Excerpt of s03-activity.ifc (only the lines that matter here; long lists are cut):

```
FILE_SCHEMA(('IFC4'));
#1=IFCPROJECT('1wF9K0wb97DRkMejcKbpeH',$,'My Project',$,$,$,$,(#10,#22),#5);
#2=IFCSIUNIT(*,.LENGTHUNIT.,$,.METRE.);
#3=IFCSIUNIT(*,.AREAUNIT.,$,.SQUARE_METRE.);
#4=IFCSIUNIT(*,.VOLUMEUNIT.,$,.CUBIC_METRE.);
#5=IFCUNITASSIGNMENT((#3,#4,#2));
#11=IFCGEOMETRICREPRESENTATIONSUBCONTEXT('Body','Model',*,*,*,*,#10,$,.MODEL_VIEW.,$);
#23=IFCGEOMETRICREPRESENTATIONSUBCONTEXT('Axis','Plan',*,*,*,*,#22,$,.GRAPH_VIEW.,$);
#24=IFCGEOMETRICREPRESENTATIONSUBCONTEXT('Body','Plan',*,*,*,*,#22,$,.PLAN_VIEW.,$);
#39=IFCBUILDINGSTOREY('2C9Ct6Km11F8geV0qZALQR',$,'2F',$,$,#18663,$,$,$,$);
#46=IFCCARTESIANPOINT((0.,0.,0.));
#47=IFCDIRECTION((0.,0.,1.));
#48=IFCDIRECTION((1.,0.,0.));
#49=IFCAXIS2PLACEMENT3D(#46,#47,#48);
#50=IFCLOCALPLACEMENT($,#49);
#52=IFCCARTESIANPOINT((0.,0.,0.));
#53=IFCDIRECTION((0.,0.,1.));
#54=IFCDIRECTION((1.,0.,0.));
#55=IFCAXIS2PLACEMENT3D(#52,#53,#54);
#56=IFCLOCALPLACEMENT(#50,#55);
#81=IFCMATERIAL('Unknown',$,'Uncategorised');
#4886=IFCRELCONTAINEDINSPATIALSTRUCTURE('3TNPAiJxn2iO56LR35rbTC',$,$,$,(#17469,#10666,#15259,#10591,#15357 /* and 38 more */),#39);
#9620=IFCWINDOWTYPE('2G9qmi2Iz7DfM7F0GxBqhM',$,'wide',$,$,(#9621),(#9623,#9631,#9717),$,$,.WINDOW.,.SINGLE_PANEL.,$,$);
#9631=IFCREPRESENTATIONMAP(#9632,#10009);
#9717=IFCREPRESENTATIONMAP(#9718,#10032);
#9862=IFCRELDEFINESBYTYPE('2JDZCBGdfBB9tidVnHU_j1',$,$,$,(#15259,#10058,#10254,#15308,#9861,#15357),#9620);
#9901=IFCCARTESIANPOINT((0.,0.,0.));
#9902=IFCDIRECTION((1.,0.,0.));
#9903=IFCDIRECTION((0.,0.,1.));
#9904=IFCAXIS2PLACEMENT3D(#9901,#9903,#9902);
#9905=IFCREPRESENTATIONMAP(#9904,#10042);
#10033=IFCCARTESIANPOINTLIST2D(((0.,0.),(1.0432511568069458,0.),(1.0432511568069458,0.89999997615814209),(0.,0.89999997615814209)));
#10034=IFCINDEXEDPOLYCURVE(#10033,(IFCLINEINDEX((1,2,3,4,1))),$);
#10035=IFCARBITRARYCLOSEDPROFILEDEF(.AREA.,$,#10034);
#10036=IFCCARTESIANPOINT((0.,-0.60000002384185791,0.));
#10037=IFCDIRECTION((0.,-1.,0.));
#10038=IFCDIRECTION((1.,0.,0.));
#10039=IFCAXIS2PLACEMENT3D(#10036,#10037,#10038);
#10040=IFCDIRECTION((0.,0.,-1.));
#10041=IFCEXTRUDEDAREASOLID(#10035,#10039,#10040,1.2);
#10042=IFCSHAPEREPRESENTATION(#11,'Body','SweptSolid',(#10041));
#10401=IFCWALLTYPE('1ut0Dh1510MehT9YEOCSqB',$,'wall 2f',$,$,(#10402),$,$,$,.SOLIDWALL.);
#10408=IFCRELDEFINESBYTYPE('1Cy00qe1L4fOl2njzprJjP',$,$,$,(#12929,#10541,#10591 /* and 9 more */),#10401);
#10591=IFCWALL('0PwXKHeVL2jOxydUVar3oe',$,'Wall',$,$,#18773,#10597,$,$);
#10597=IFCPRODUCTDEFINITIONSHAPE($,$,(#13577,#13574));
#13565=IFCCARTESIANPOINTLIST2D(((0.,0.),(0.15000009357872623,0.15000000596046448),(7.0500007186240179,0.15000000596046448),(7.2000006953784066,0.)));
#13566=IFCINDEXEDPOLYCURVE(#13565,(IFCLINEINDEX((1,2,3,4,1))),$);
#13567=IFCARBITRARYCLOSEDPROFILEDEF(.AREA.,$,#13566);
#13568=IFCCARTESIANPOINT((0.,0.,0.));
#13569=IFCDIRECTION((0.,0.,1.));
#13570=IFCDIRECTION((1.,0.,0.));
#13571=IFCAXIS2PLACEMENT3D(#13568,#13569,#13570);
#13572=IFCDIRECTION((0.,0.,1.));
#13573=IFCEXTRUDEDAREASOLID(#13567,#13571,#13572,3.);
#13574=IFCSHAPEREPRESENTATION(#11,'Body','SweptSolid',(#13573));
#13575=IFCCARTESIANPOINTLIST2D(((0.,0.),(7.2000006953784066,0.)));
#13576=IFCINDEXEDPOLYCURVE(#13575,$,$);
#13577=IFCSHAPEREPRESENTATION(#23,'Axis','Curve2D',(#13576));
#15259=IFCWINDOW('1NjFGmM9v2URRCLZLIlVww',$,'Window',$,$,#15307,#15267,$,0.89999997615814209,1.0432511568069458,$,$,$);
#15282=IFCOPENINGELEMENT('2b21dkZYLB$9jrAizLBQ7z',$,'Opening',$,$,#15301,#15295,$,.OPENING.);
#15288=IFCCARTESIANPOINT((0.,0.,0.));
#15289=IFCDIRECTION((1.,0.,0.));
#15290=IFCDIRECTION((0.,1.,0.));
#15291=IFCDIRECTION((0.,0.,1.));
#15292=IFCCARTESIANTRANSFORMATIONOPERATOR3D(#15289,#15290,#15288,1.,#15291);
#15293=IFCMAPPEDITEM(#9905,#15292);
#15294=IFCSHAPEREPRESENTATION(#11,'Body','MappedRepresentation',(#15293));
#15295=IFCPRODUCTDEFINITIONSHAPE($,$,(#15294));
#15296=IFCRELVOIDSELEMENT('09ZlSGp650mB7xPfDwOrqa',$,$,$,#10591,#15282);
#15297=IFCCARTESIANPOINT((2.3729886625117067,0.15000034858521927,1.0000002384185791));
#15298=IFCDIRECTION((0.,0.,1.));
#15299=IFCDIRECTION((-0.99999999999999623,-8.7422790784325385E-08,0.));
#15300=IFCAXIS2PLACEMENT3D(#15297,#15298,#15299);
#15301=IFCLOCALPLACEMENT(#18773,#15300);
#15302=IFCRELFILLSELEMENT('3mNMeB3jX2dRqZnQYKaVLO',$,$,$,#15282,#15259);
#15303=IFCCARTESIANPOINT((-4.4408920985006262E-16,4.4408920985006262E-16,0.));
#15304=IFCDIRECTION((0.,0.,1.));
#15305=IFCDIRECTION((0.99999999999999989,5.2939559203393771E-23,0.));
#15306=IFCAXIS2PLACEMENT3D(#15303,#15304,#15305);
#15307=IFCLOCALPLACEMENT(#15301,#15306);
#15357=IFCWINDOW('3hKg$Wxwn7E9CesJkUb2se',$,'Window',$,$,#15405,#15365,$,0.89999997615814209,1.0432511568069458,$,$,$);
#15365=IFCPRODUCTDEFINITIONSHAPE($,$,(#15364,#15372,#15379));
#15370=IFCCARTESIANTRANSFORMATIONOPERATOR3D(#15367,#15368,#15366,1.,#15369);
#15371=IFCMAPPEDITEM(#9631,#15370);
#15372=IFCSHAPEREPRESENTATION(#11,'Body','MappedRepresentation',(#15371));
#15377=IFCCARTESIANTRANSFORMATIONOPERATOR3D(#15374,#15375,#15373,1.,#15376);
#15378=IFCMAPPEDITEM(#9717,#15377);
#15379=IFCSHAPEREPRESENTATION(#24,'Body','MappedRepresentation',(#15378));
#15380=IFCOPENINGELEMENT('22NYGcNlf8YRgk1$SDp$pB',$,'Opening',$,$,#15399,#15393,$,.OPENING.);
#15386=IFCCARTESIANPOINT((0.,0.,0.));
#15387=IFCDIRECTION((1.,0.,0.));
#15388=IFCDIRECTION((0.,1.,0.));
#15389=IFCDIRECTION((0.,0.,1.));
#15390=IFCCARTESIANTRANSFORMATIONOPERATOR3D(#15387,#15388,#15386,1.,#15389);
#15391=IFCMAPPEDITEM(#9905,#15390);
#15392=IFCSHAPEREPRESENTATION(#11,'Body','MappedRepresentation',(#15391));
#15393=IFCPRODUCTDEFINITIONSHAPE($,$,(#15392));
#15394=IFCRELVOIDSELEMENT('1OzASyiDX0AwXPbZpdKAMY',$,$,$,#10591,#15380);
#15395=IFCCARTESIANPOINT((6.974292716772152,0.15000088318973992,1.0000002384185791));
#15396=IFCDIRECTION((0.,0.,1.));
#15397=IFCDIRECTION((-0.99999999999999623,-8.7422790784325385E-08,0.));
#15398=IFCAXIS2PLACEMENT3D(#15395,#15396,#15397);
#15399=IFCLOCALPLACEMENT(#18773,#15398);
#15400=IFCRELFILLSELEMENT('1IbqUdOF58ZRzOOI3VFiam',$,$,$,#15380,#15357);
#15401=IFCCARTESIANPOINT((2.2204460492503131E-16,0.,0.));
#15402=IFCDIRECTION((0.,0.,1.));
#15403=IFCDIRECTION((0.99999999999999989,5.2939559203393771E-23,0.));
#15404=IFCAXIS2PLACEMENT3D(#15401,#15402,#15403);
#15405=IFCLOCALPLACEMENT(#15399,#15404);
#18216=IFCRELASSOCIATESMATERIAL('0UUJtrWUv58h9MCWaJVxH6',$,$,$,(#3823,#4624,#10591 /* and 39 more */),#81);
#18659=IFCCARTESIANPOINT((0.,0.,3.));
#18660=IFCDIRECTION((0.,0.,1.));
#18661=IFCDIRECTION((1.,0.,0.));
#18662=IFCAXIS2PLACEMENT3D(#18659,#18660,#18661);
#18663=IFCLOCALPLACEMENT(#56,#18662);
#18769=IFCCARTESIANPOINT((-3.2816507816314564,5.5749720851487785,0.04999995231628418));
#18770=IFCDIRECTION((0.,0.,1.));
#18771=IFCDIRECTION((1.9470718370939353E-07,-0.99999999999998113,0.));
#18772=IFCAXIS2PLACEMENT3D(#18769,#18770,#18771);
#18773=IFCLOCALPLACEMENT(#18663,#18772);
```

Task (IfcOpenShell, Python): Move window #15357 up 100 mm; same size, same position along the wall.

```python
import numpy as np
import ifcopenshell
import ifcopenshell.api.geometry
import ifcopenshell.util.placement
import ifcopenshell.util.unit

model = ifcopenshell.open("s03-activity.ifc")
unit_scale = ifcopenshell.util.unit.calculate_unit_scale(model)

window = model.by_id(15357)
opening = window.FillsVoids[0].RelatingOpeningElement
dz = 0.1

shift = np.array([0.0, 0.0, dz])
# The window is placed relative to its opening, so it follows when the opening moves.
matrix = ifcopenshell.util.placement.get_local_placement(opening.ObjectPlacement)
matrix[:3, 3] += shift
ifcopenshell.api.geometry.edit_object_placement(
    model, product=opening, matrix=matrix, is_si=False, should_transform_children=True
)

print(f"moved by {dz * unit_scale:+.3f} m")

model.write("s03-activity_updated.ifc")
```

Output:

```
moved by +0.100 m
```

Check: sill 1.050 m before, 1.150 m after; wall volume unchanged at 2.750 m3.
